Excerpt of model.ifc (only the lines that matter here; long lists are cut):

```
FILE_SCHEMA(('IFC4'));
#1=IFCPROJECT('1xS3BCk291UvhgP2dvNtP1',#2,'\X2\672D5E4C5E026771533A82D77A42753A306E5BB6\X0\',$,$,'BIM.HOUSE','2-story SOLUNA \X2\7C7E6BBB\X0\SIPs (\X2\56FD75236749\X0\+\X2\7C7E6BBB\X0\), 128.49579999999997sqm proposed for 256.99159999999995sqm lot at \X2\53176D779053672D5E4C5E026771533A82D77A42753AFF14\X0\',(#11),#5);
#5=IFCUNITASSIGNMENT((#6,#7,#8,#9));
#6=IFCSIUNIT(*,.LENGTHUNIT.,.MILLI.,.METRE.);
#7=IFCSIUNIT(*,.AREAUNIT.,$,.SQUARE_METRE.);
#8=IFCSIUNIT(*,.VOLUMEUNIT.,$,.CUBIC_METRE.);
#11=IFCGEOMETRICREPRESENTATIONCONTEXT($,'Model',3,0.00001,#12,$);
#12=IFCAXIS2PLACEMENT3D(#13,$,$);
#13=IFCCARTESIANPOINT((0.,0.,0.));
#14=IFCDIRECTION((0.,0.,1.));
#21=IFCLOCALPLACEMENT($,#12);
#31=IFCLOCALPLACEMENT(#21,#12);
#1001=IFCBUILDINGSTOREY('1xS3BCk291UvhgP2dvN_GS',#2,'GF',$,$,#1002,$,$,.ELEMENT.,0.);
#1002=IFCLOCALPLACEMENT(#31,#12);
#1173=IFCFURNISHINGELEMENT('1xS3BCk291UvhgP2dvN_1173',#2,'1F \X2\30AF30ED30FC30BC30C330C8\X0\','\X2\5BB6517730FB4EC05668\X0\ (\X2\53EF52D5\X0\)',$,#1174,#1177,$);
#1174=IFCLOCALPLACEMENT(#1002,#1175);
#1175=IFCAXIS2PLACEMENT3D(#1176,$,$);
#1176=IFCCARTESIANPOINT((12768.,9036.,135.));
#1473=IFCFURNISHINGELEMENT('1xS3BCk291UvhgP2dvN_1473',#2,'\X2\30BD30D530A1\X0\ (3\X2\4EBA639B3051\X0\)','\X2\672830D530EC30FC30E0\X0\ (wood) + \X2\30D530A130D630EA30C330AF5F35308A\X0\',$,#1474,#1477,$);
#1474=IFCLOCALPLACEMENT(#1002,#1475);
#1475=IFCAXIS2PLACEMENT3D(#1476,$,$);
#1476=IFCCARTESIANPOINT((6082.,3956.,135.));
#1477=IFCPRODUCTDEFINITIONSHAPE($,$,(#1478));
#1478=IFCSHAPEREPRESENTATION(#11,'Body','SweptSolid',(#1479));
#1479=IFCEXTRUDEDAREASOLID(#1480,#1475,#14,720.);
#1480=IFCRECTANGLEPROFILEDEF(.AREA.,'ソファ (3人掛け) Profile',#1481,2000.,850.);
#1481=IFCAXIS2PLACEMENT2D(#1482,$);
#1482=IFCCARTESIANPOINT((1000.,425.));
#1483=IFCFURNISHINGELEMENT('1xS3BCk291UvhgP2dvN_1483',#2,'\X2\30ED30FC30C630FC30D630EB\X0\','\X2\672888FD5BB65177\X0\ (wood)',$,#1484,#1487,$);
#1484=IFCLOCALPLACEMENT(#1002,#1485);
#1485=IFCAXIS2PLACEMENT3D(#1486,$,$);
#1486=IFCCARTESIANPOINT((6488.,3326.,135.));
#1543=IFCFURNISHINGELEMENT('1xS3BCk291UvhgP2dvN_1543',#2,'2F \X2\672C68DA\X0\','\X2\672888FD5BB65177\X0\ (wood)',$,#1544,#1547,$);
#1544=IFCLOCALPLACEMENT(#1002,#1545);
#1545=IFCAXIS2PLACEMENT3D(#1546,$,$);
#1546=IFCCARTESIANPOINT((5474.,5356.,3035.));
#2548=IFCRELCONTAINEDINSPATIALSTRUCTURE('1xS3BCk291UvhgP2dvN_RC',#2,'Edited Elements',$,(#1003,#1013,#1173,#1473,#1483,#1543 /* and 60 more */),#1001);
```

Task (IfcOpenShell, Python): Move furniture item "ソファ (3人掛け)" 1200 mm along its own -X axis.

```python
import ifcopenshell
import ifcopenshell.api.geometry
import ifcopenshell.util.placement

model = ifcopenshell.open("model.ifc")

item = model.by_guid("1xS3BCk291UvhgP2dvN_1473")
matrix = ifcopenshell.util.placement.get_local_placement(item.ObjectPlacement)
matrix[:3, 3] -= matrix[:3, 0] * 1200.0
ifcopenshell.api.geometry.edit_object_placement(model, product=item, matrix=matrix, is_si=False)

print(ifcopenshell.util.placement.get_local_placement(item.ObjectPlacement).round(3) + 0.0)

model.write("model-out.ifc")
```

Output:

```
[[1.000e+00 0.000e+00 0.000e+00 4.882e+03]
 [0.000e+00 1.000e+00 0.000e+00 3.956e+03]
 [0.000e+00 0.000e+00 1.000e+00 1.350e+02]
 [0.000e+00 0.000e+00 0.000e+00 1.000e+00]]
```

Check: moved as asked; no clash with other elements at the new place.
